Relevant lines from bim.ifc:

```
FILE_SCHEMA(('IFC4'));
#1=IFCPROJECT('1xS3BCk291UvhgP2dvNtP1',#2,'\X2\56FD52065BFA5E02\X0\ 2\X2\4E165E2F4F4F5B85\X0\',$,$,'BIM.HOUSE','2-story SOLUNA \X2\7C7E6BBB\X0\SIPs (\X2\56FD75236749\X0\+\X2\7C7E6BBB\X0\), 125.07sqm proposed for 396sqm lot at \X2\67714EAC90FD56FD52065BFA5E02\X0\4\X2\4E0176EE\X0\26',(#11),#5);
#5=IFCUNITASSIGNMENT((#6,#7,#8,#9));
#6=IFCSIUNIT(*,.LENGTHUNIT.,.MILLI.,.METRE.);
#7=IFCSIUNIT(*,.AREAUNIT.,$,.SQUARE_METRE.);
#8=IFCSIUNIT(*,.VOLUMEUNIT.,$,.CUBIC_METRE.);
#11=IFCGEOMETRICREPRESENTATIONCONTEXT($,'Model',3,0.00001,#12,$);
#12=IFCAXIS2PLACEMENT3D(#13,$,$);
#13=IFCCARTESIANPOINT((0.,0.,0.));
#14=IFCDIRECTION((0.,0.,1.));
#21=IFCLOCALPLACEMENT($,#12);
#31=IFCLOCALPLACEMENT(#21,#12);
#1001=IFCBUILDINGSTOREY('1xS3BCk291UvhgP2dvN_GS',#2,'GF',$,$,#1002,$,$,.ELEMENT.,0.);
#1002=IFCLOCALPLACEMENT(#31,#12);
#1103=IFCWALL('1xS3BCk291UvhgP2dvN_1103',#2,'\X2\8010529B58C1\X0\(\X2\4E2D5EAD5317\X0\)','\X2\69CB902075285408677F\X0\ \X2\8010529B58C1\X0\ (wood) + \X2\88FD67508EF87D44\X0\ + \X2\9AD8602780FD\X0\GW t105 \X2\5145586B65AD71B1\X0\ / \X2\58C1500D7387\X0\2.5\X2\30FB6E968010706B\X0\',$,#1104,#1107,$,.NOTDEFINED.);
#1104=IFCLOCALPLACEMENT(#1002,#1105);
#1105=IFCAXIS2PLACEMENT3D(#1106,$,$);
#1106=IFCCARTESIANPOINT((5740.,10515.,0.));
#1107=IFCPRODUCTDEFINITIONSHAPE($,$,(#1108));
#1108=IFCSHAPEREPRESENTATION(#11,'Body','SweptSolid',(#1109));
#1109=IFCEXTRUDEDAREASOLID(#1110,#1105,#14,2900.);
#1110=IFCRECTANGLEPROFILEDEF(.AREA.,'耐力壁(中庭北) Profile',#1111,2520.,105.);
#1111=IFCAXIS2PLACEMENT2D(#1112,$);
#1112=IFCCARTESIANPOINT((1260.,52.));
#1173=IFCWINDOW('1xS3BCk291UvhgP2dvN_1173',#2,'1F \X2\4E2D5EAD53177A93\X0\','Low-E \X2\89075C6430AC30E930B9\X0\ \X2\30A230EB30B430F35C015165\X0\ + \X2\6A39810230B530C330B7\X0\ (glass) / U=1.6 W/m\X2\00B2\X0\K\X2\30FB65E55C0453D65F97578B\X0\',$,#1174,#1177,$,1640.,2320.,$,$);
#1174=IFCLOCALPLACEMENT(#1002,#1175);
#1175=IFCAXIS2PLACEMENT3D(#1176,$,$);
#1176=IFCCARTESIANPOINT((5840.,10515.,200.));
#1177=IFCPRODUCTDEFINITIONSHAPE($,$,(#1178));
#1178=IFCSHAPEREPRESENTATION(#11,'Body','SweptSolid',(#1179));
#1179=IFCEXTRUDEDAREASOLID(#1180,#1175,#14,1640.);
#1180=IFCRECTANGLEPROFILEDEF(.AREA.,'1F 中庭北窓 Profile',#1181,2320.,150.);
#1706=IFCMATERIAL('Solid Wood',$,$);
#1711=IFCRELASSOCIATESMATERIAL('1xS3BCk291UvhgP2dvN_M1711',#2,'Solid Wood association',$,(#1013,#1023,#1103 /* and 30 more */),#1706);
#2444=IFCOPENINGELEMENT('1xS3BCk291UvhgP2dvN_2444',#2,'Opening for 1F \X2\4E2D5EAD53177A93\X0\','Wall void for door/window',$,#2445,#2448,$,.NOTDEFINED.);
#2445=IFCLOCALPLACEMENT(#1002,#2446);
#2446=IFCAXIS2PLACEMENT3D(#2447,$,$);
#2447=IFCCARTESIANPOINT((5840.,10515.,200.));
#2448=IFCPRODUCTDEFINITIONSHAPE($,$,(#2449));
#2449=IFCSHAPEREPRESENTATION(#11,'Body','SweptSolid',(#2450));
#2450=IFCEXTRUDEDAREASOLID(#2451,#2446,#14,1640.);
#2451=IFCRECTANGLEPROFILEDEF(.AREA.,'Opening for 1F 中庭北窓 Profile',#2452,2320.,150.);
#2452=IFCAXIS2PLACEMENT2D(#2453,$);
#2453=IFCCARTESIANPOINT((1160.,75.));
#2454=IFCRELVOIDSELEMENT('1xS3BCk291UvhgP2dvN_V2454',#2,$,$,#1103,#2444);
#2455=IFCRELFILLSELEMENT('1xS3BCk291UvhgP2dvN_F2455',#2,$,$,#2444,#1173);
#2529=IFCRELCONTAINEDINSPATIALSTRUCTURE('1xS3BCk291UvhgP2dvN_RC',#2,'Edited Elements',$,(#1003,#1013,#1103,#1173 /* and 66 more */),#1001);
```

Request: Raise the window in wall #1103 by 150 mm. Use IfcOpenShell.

```python
import numpy as np
import ifcopenshell
import ifcopenshell.api.geometry
import ifcopenshell.util.placement
import ifcopenshell.util.unit

model = ifcopenshell.open("bim.ifc")
unit_scale = ifcopenshell.util.unit.calculate_unit_scale(model)

window = model.by_guid("1xS3BCk291UvhgP2dvN_1173")
opening = window.FillsVoids[0].RelatingOpeningElement
dz = 150.0

shift = np.array([0.0, 0.0, dz])
# The window is not placed relative to its opening, so move both.
for product in (opening, window):
    matrix = ifcopenshell.util.placement.get_local_placement(product.ObjectPlacement)
    matrix[:3, 3] += shift
    ifcopenshell.api.geometry.edit_object_placement(model, product=product, matrix=matrix, is_si=False)

print(f"moved by {dz * unit_scale:+.3f} m")

model.write("bim_edited.ifc")
```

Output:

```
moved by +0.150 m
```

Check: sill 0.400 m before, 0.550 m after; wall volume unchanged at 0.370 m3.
